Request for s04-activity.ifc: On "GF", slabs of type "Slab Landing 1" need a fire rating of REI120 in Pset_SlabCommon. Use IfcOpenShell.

First a look at what the model holds.

```python
import ifcopenshell
import ifcopenshell.util.element

model = ifcopenshell.open("s04-activity.ifc")
print(model.schema)
storey = next(s for s in model.by_type("IfcBuildingStorey") if s.Name == "GF")
slabs = [e for e in ifcopenshell.util.element.get_decomposition(storey) if e.is_a("IfcSlab")]
seen = {}
for e in slabs:
    element_type = ifcopenshell.util.element.get_type(e)
    key = (element_type.Name if element_type != e and element_type else None, ifcopenshell.util.element.get_pset(e, "Pset_SlabCommon", "FireRating"))
    seen[key] = seen.get(key, 0) + 1
for (name, value), count in sorted(seen.items(), key=str):
    print(count, "x", name, "|", value)
```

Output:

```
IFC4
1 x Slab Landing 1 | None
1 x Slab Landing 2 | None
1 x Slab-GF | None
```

```python
import ifcopenshell
import ifcopenshell.api.pset
import ifcopenshell.util.element

model = ifcopenshell.open("s04-activity.ifc")

storey = next(s for s in model.by_type("IfcBuildingStorey") if s.Name == "GF")
slabs = [e for e in ifcopenshell.util.element.get_decomposition(storey) if e.is_a("IfcSlab")]

count = 0
for e in slabs:
    element_type = ifcopenshell.util.element.get_type(e)
    if element_type in (None, e) or element_type.Name != "Slab Landing 1":
        continue
    # add_pset returns the element's existing set when there is one.
    pset = ifcopenshell.api.pset.add_pset(model, product=e, name="Pset_SlabCommon")
    ifcopenshell.api.pset.edit_pset(model, pset=pset, properties={"FireRating": "REI120"})
    count += 1

print(count, "slabs updated")

model.write("s04-activity-out.ifc")
```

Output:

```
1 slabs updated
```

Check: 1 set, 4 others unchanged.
